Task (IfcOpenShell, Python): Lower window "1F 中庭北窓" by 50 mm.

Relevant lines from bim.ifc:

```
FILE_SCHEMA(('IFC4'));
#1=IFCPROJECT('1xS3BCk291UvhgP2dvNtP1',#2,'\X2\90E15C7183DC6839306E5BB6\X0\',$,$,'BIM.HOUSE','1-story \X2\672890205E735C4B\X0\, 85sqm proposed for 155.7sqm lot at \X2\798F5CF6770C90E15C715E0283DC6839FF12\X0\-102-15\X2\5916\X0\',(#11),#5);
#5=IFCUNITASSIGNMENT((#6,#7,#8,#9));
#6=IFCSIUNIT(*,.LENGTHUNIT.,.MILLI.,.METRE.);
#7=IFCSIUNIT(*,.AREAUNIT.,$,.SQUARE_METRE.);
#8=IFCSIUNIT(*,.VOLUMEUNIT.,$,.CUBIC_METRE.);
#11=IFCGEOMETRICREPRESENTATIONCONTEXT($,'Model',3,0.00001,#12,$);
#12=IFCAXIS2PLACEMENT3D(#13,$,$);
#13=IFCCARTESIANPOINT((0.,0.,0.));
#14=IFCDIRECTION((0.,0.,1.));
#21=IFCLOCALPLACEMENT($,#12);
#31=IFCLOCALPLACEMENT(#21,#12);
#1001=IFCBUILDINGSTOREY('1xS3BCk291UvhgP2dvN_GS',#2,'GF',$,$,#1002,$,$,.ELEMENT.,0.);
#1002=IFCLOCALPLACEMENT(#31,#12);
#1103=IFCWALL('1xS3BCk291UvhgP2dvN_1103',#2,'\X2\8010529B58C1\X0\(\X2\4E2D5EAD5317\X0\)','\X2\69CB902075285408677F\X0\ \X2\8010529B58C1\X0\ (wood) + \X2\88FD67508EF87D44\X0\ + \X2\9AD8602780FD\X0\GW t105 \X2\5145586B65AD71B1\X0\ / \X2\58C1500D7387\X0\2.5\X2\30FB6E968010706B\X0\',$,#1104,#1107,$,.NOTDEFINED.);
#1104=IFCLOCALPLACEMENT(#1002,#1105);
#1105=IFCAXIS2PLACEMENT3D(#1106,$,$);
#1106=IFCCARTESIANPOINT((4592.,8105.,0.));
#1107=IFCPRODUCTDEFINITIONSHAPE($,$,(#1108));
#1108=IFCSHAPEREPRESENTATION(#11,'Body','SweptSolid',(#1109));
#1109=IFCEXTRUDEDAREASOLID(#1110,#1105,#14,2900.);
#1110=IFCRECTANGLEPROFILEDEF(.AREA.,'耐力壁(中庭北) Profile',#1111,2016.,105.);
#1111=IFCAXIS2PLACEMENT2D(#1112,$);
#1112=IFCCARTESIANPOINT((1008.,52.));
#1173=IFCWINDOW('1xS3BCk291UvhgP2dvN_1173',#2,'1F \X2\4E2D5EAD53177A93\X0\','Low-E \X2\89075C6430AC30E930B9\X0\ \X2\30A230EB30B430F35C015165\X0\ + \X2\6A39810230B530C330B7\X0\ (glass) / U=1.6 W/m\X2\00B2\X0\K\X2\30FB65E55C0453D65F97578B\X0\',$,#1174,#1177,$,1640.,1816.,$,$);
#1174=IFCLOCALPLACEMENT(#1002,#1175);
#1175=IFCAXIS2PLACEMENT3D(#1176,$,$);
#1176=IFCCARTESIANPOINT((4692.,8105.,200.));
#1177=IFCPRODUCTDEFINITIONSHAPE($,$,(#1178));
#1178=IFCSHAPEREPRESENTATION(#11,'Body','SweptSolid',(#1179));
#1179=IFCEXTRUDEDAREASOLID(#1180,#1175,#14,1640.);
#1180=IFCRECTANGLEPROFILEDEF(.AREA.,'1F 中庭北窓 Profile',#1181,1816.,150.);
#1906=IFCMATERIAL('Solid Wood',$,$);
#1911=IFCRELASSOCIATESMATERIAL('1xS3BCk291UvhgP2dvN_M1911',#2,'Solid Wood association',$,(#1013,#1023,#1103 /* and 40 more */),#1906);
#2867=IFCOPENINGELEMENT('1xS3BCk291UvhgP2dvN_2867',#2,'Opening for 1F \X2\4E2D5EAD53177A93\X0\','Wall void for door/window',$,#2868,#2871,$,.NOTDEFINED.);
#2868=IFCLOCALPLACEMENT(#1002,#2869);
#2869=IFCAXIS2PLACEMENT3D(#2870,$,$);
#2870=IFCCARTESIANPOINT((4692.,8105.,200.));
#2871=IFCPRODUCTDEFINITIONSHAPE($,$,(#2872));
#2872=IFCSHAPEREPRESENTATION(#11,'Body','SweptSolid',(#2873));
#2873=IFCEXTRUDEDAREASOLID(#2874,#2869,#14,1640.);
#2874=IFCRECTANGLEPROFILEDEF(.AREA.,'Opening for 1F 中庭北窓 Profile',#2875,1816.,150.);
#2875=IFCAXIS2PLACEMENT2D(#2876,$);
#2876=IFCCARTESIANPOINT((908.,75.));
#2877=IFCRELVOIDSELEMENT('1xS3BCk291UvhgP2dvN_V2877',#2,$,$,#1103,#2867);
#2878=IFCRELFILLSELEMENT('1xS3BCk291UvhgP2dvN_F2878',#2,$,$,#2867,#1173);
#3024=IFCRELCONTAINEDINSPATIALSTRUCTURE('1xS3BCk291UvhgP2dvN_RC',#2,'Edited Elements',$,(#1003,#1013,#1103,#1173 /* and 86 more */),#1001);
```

```python
import numpy as np
import ifcopenshell
import ifcopenshell.api.geometry
import ifcopenshell.util.placement
import ifcopenshell.util.unit

model = ifcopenshell.open("bim.ifc")
unit_scale = ifcopenshell.util.unit.calculate_unit_scale(model)

window = model.by_id(1173)
opening = window.FillsVoids[0].RelatingOpeningElement
dz = -50.0

shift = np.array([0.0, 0.0, dz])
# The window is not placed relative to its opening, so move both.
for product in (opening, window):
    matrix = ifcopenshell.util.placement.get_local_placement(product.ObjectPlacement)
    matrix[:3, 3] += shift
    ifcopenshell.api.geometry.edit_object_placement(model, product=product, matrix=matrix, is_si=False)

print(f"moved by {dz * unit_scale:+.3f} m")

model.write("bim_v2.ifc")
```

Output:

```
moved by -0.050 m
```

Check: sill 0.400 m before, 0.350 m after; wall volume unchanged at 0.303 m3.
